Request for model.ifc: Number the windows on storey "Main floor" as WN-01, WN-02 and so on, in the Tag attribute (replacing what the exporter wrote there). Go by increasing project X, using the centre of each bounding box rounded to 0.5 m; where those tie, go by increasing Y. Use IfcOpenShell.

First a look at what the model holds.

```python
import ifcopenshell
import ifcopenshell.util.element
import ifcopenshell.util.placement

model = ifcopenshell.open("model.ifc")
print(model.schema)
storey = next(s for s in model.by_type("IfcBuildingStorey") if s.Name == "Main floor")
windows = [e for e in ifcopenshell.util.element.get_decomposition(storey) if e.is_a("IfcWindow")]
for e in sorted(windows, key=lambda e: e.id()):
    origin = ifcopenshell.util.placement.get_local_placement(e.ObjectPlacement)[:3, 3]
    print(e.id(), e.Tag, e.Name, origin.round(2) + 0.0, sep=" | ")
```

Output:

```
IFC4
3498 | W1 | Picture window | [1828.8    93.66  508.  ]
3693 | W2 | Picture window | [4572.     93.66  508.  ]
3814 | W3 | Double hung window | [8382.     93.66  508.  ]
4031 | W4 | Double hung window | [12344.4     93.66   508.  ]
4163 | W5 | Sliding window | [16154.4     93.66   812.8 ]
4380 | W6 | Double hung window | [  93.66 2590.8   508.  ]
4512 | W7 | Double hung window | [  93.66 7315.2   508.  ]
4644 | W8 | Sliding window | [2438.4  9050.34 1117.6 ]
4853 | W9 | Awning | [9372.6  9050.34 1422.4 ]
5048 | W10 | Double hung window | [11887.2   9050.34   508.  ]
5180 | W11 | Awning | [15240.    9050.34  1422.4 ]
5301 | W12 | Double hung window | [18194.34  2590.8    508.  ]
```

```python
import ifcopenshell
import ifcopenshell.geom
import ifcopenshell.util.element
import ifcopenshell.util.shape

model = ifcopenshell.open("model.ifc")
settings = ifcopenshell.geom.settings()
settings.set("use-world-coords", True)


def centre(element):
    shape = ifcopenshell.geom.create_shape(settings, element)
    return ifcopenshell.util.shape.get_bbox_centroid(shape.geometry)


storey = next(s for s in model.by_type("IfcBuildingStorey") if s.Name == "Main floor")
windows = [e for e in ifcopenshell.util.element.get_decomposition(storey) if e.is_a("IfcWindow")]

# Insertion points can sit at a corner or the storey origin, so sort by the geometry (in metres).
centres = {e: centre(e) for e in windows}
windows.sort(key=lambda e: (round(centres[e][0] / 0.5), centres[e][1]))

for i, e in enumerate(windows, start=1):
    number = f"WN-{i:02d}"
    e.Tag = number
    print(e.id(), number)

model.write("model_rev.ifc")
```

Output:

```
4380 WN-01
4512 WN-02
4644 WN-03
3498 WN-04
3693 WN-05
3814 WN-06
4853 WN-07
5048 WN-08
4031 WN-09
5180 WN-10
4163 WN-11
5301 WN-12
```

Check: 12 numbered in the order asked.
